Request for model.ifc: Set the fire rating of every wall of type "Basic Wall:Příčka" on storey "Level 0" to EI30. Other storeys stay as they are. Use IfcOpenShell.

First a look at what the model holds.

```python
import ifcopenshell
import ifcopenshell.util.element

model = ifcopenshell.open("model.ifc")
print(model.schema)
storey = next(s for s in model.by_type("IfcBuildingStorey") if s.Name == "Level 0")
walls = [e for e in ifcopenshell.util.element.get_decomposition(storey) if e.is_a("IfcWall")]
seen = {}
for e in walls:
    element_type = ifcopenshell.util.element.get_type(e)
    key = (element_type.Name if element_type != e and element_type else None, ifcopenshell.util.element.get_pset(e, "Pset_WallCommon", "FireRating"))
    seen[key] = seen.get(key, 0) + 1
for (name, value), count in sorted(seen.items(), key=str):
    print(count, "x", name, "|", value)
```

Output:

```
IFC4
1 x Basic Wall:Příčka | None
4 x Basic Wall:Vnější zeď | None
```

```python
import ifcopenshell
import ifcopenshell.api.pset
import ifcopenshell.util.element

model = ifcopenshell.open("model.ifc")

storey = next(s for s in model.by_type("IfcBuildingStorey") if s.Name == "Level 0")
walls = [e for e in ifcopenshell.util.element.get_decomposition(storey) if e.is_a("IfcWall")]

count = 0
for e in walls:
    element_type = ifcopenshell.util.element.get_type(e)
    if element_type in (None, e) or element_type.Name != "Basic Wall:Příčka":
        continue
    # add_pset returns the element's existing set when there is one.
    pset = ifcopenshell.api.pset.add_pset(model, product=e, name="Pset_WallCommon")
    ifcopenshell.api.pset.edit_pset(model, pset=pset, properties={"FireRating": "EI30"})
    count += 1

print(count, "walls updated")

model.write("model_rev.ifc")
```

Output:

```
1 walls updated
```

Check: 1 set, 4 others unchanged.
